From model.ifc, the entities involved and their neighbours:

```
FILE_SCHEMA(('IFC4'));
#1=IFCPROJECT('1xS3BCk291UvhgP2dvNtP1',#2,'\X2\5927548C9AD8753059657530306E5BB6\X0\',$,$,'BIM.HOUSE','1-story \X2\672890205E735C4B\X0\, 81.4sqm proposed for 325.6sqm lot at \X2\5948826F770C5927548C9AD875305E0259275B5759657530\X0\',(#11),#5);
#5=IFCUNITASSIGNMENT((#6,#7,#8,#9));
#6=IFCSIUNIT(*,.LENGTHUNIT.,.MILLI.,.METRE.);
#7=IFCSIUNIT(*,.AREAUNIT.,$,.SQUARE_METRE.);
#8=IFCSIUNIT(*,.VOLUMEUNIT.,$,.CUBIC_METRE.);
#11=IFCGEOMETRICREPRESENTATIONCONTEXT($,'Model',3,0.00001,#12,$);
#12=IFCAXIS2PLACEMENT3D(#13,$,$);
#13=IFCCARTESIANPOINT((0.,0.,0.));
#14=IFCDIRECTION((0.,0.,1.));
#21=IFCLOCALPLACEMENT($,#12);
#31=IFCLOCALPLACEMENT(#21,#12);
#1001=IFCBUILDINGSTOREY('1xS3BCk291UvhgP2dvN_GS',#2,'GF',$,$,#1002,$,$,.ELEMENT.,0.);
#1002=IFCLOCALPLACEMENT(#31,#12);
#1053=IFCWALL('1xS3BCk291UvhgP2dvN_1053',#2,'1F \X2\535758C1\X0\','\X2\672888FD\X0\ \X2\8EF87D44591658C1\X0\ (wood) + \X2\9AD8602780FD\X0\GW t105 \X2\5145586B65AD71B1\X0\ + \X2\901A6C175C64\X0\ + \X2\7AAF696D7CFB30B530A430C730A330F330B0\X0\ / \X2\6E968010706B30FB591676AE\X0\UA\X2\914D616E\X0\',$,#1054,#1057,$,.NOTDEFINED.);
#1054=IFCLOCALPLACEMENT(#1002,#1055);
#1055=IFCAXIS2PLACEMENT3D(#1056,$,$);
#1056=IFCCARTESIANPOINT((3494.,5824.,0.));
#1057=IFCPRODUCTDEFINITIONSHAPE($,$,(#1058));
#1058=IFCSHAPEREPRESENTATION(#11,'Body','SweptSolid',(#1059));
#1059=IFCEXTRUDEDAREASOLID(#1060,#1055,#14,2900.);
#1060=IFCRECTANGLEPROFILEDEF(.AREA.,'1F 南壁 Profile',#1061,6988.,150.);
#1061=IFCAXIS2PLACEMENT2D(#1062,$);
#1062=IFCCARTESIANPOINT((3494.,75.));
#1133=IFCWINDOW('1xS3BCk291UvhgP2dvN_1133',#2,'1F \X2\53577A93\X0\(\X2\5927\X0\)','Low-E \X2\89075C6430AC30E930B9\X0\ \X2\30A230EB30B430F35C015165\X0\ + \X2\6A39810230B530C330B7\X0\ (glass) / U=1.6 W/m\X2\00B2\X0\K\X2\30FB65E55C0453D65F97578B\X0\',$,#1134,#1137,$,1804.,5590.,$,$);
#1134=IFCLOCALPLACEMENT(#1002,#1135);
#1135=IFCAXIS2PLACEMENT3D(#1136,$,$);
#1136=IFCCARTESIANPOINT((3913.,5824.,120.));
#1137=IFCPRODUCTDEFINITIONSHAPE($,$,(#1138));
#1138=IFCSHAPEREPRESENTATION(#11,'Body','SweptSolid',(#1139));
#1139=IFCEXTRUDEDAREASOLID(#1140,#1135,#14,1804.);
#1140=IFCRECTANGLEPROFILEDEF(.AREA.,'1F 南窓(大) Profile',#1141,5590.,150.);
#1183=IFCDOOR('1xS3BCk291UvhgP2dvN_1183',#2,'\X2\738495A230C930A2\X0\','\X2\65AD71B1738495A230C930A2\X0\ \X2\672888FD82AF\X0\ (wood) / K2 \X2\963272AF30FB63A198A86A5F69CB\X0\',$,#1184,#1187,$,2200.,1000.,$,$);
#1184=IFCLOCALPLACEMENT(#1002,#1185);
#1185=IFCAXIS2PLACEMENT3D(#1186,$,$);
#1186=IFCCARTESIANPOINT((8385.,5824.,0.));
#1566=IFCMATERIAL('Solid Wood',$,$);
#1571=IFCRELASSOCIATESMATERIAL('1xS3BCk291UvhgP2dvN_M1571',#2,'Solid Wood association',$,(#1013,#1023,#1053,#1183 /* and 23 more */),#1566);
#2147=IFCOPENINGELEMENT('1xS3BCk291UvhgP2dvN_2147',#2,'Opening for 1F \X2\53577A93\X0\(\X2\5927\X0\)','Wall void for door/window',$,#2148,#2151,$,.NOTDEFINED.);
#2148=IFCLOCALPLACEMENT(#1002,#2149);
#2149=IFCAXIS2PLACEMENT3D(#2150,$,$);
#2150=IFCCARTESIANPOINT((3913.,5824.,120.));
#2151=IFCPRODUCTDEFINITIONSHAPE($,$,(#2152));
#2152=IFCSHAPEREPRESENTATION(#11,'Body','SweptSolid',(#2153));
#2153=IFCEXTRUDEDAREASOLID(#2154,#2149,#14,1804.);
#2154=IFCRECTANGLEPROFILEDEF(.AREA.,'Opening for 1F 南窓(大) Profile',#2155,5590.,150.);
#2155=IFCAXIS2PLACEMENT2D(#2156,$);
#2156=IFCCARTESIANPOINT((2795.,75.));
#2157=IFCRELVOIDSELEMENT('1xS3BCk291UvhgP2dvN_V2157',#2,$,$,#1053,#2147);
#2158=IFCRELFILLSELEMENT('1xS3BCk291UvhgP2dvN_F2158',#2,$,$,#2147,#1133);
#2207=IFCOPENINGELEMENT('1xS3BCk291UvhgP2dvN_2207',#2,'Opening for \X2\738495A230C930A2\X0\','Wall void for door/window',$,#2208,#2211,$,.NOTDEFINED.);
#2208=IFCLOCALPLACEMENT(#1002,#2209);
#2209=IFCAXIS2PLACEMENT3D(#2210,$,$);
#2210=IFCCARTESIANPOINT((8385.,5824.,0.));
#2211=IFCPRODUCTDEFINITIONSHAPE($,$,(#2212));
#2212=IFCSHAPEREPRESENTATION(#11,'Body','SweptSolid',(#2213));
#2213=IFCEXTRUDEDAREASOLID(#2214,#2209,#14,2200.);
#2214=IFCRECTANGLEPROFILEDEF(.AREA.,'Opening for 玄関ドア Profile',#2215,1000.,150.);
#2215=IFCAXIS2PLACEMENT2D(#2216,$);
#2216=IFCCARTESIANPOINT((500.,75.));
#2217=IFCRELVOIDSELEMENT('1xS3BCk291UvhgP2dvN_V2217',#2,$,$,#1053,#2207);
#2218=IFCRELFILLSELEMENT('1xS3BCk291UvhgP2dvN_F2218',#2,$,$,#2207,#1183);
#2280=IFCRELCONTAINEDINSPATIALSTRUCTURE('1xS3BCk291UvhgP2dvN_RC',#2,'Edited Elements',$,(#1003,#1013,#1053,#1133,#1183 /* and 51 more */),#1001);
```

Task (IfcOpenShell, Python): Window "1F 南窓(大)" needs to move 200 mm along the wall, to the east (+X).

```python
import ifcopenshell
import ifcopenshell.api.geometry
import ifcopenshell.util.placement
import ifcopenshell.util.unit

model = ifcopenshell.open("model.ifc")
unit_scale = ifcopenshell.util.unit.calculate_unit_scale(model)

window = model.by_id(1133)
opening = window.FillsVoids[0].RelatingOpeningElement
wall = opening.VoidsElements[0].RelatingBuildingElement

wall_matrix = ifcopenshell.util.placement.get_local_placement(wall.ObjectPlacement)
shift = wall_matrix[:3, 0] * 0.2 / unit_scale
before = ifcopenshell.util.placement.get_local_placement(window.ObjectPlacement)[:3, 3].copy()

# The window is not placed relative to its opening, so move both.
for product in (opening, window):
    matrix = ifcopenshell.util.placement.get_local_placement(product.ObjectPlacement)
    matrix[:3, 3] += shift
    ifcopenshell.api.geometry.edit_object_placement(model, product=product, matrix=matrix, is_si=False)

after = ifcopenshell.util.placement.get_local_placement(window.ObjectPlacement)[:3, 3]
print("window moved by", (after - before).round(3) + 0.0)

model.write("model_v2.ifc")
```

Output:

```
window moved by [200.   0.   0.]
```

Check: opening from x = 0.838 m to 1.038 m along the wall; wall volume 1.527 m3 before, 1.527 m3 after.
